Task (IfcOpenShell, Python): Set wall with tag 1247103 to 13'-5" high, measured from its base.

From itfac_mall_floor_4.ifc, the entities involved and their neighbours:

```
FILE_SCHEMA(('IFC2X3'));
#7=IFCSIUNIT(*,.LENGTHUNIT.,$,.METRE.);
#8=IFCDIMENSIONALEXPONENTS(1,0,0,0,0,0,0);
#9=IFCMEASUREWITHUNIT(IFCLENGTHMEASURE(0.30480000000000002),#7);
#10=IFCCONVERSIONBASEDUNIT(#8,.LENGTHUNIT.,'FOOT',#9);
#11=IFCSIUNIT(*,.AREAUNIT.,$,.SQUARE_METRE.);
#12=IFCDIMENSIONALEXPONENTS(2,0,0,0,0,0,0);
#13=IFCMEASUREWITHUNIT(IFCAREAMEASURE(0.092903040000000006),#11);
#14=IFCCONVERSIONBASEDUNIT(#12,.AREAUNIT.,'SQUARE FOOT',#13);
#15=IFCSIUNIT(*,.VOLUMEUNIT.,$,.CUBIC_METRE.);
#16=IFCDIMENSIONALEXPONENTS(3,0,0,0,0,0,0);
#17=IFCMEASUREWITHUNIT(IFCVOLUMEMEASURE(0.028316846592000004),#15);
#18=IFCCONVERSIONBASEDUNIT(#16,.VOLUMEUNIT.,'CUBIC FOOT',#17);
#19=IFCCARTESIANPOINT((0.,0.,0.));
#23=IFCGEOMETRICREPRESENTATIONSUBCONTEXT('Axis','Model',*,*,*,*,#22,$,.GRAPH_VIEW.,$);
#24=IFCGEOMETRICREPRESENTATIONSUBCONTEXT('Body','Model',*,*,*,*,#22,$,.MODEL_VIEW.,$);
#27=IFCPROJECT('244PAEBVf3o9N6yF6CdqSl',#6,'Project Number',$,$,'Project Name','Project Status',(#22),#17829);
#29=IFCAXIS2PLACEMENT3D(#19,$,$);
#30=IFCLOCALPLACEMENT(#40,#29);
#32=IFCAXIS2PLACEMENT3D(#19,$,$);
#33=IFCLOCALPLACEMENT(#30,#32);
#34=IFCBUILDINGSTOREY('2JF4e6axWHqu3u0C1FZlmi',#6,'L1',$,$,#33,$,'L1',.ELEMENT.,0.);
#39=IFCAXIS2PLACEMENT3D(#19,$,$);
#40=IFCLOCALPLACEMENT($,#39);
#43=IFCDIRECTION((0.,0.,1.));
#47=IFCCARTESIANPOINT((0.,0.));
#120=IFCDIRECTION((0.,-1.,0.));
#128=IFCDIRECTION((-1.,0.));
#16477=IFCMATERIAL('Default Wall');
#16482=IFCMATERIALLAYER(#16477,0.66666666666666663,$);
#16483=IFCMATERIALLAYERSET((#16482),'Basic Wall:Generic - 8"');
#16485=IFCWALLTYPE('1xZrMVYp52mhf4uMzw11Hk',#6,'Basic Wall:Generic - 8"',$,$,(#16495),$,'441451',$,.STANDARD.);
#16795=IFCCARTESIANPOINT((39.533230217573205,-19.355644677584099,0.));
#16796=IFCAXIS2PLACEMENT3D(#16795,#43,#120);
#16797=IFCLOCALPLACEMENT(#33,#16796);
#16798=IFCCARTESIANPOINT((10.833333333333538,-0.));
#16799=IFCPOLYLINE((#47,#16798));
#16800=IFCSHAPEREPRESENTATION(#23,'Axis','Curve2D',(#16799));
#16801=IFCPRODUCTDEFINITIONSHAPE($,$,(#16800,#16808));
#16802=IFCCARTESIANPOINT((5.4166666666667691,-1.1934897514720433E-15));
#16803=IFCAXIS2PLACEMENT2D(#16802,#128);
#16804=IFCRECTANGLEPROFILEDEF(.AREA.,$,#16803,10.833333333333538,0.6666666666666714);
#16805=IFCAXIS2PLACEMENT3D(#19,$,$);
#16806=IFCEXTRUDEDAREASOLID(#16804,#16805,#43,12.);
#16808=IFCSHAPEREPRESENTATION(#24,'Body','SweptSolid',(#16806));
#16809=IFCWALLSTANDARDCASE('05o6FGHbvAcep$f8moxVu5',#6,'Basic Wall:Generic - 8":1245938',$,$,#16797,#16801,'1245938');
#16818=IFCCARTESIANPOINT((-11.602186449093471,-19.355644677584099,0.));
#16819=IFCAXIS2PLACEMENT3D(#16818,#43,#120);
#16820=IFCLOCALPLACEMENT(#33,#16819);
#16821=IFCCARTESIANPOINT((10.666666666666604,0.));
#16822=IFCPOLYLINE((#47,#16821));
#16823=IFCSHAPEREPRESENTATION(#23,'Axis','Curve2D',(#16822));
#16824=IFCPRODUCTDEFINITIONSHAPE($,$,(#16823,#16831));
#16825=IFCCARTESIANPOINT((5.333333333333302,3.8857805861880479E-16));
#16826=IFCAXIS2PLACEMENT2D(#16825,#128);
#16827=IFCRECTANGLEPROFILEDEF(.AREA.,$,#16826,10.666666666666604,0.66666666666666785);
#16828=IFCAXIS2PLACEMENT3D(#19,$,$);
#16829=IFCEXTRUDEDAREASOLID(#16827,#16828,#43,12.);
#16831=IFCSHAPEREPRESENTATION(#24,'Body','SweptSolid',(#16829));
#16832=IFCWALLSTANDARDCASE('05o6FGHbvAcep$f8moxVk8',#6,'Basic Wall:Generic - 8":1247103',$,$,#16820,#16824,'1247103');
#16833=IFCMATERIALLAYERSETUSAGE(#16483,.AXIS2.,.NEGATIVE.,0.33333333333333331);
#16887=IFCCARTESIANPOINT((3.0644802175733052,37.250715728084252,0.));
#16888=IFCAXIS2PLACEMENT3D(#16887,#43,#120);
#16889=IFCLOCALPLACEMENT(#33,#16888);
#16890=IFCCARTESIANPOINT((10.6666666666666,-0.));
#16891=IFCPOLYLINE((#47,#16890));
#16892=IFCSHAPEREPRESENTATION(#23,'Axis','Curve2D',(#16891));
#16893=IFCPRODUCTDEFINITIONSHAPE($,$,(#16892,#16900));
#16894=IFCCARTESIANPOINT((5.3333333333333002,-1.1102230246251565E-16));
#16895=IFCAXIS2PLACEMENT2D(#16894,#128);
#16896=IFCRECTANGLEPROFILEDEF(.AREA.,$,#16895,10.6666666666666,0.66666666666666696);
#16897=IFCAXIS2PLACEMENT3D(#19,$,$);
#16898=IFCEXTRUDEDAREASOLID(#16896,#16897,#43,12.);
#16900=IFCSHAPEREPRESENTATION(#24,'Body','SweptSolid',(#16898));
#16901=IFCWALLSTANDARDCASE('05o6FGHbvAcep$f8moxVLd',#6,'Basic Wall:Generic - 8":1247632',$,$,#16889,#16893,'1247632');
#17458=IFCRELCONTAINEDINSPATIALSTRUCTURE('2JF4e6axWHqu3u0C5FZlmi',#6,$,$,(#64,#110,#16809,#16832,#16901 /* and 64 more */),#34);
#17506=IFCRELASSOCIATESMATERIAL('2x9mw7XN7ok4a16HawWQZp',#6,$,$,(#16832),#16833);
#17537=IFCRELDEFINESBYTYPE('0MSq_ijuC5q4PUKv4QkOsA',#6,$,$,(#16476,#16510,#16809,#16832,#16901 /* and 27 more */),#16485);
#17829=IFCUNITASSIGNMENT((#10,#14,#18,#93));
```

```python
import ifcopenshell
import ifcopenshell.geom
import ifcopenshell.util.representation
import ifcopenshell.util.shape
import ifcopenshell.util.unit

model = ifcopenshell.open("itfac_mall_floor_4.ifc")
unit_scale = ifcopenshell.util.unit.calculate_unit_scale(model)
settings = ifcopenshell.geom.settings()


def volume(element):
    """Net volume in cubic metres, openings subtracted."""
    shape = ifcopenshell.geom.create_shape(settings, element)
    return ifcopenshell.util.shape.get_volume(shape.geometry)


wall = model.by_guid("05o6FGHbvAcep$f8moxVk8")
before = volume(wall)

body = ifcopenshell.util.representation.get_representation(wall, "Model", "Body")
solid = body.Items[0]
old_height = solid.Depth
solid.Depth = 161 * 0.0254 / unit_scale
after = volume(wall)

print(f"height {old_height:g} -> {solid.Depth:g}, volume {before:.3f} -> {after:.3f} m3")

model.write("itfac_mall_floor_4_v2.ifc")
```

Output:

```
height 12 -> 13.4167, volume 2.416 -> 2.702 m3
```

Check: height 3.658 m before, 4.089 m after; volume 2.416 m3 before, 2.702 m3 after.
